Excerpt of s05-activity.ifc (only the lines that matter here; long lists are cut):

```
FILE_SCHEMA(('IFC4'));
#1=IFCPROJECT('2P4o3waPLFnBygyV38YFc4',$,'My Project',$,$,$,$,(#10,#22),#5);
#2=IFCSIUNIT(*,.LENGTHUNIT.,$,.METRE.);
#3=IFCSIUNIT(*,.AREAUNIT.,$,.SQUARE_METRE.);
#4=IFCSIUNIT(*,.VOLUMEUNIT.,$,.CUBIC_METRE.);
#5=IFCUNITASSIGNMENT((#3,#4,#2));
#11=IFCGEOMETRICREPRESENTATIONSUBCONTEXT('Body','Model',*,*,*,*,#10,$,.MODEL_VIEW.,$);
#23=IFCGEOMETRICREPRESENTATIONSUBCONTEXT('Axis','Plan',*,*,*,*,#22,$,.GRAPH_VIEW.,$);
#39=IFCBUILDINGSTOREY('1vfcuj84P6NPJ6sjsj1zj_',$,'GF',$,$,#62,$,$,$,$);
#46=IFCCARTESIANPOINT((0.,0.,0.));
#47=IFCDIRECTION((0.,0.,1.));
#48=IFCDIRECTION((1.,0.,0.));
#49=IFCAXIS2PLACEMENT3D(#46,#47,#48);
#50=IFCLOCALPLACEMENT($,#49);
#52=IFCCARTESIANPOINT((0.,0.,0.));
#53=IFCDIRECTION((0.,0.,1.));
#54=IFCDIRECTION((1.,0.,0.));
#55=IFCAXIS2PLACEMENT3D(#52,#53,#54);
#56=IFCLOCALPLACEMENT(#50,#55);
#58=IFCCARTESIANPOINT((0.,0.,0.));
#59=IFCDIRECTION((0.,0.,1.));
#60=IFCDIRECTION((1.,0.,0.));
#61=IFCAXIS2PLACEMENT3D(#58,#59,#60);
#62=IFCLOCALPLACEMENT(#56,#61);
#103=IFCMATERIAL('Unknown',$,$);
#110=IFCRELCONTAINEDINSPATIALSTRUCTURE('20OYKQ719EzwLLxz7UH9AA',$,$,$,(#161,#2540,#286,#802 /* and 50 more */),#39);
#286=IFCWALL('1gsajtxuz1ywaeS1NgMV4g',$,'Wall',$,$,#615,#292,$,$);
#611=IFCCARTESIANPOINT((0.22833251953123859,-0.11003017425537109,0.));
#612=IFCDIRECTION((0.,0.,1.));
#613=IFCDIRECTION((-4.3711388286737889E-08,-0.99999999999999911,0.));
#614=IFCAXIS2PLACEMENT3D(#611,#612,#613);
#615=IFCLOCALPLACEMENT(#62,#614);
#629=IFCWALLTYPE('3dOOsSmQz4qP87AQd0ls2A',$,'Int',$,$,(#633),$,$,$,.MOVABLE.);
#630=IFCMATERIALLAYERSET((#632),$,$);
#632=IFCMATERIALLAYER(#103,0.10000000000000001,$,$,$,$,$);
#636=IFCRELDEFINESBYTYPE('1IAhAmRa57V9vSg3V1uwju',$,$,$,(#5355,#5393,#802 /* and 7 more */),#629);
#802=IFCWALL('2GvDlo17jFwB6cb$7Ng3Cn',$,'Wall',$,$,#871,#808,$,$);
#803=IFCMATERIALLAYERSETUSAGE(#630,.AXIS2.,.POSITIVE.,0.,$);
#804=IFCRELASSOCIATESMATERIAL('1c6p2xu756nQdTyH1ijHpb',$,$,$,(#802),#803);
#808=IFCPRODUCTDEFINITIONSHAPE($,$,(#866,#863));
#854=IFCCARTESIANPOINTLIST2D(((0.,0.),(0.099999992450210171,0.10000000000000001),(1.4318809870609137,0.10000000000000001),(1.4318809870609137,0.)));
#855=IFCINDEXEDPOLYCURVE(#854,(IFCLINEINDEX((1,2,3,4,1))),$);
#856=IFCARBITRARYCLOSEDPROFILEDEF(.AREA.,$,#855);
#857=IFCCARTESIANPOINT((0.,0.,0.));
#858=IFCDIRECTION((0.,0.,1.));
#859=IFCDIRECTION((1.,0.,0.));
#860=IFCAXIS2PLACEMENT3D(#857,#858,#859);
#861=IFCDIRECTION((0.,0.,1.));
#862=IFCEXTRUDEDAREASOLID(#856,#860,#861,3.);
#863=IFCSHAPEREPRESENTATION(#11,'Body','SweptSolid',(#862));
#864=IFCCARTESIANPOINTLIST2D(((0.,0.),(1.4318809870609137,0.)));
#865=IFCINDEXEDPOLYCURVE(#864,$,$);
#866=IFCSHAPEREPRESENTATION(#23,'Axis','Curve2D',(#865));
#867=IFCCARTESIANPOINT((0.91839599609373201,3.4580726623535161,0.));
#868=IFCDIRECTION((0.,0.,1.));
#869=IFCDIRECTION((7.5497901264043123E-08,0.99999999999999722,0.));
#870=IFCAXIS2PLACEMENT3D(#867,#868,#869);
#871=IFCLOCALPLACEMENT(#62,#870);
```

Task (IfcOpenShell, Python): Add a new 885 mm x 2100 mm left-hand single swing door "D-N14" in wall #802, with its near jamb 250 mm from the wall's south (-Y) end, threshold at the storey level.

```python
import numpy as np
import ifcopenshell
import ifcopenshell.api.feature
import ifcopenshell.api.geometry
import ifcopenshell.api.root
import ifcopenshell.api.spatial
import ifcopenshell.geom
import ifcopenshell.util.element
import ifcopenshell.util.placement
import ifcopenshell.util.representation
import ifcopenshell.util.shape
import ifcopenshell.util.unit

model = ifcopenshell.open("s05-activity.ifc")
unit_scale = ifcopenshell.util.unit.calculate_unit_scale(model)
settings = ifcopenshell.geom.settings()


def volume(element):
    """Net volume in cubic metres, openings subtracted."""
    shape = ifcopenshell.geom.create_shape(settings, element)
    return ifcopenshell.util.shape.get_volume(shape.geometry)


wall = model.by_id(802)
storey = ifcopenshell.util.element.get_container(wall, ifc_class="IfcBuildingStorey")
context = ifcopenshell.util.representation.get_context(model, "Model", "Body", "MODEL_VIEW")
before = volume(wall)

width, height, from_end, sill = 0.885, 2.1, 0.25, 0.0  # metres

# The wall runs along its own X axis, and the end named is its -X end.
wall_shape = ifcopenshell.geom.create_shape(settings, wall)
x, y, z = ifcopenshell.util.shape.get_vertices(wall_shape.geometry).T
start = x.min() + from_end
face, thickness = float(y.min()), float(y.max() - y.min())
wall_matrix = ifcopenshell.util.placement.get_local_placement(wall.ObjectPlacement)
level = ifcopenshell.util.placement.get_local_placement(storey.ObjectPlacement)[2, 3]


def in_wall(x, y):
    """Placement at x, y metres in the wall's axes, at sill height."""
    matrix = wall_matrix.copy()
    matrix[:, 3] = wall_matrix @ np.array([x / unit_scale, y / unit_scale, 0.0, 1.0])
    matrix[2, 3] = level + sill / unit_scale
    return matrix


# Opening: a box that overshoots both wall faces by 50 mm.
opening = ifcopenshell.api.root.create_entity(model, ifc_class="IfcOpeningElement", predefined_type="OPENING")
box = ifcopenshell.api.geometry.add_wall_representation(
    model, context=context, length=width, height=height, thickness=thickness + 0.1
)
ifcopenshell.api.geometry.assign_representation(model, product=opening, representation=box)
ifcopenshell.api.geometry.edit_object_placement(model, product=opening, matrix=in_wall(start, face - 0.05), is_si=False)
ifcopenshell.api.feature.add_feature(model, feature=opening, element=wall)

door = ifcopenshell.api.root.create_entity(model, ifc_class="IfcDoor", name="D-N14", predefined_type="DOOR")
door.OverallWidth, door.OverallHeight = width / unit_scale, height / unit_scale
door.OperationType = "SINGLE_SWING_LEFT"
body = ifcopenshell.api.geometry.add_door_representation(
    model,
    context=context,
    overall_width=door.OverallWidth,
    overall_height=door.OverallHeight,
    operation_type="SINGLE_SWING_LEFT",
    lining_properties={"LiningDepth": thickness / unit_scale, "ThresholdDepth": thickness / unit_scale},
)
ifcopenshell.api.geometry.assign_representation(model, product=door, representation=body)
ifcopenshell.api.spatial.assign_container(model, products=[door], relating_structure=storey)
ifcopenshell.api.feature.add_filling(model, opening=opening, element=door)

# The lining spans the wall, so the door starts at the wall face.
ifcopenshell.api.geometry.edit_object_placement(model, product=door, matrix=in_wall(start, face), is_si=False)

after = volume(wall)

print(f"wall volume {before:.3f} -> {after:.3f} m3")

model.write("s05-activity_updated.ifc")
```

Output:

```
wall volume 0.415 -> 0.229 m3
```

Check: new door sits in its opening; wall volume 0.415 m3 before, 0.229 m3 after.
